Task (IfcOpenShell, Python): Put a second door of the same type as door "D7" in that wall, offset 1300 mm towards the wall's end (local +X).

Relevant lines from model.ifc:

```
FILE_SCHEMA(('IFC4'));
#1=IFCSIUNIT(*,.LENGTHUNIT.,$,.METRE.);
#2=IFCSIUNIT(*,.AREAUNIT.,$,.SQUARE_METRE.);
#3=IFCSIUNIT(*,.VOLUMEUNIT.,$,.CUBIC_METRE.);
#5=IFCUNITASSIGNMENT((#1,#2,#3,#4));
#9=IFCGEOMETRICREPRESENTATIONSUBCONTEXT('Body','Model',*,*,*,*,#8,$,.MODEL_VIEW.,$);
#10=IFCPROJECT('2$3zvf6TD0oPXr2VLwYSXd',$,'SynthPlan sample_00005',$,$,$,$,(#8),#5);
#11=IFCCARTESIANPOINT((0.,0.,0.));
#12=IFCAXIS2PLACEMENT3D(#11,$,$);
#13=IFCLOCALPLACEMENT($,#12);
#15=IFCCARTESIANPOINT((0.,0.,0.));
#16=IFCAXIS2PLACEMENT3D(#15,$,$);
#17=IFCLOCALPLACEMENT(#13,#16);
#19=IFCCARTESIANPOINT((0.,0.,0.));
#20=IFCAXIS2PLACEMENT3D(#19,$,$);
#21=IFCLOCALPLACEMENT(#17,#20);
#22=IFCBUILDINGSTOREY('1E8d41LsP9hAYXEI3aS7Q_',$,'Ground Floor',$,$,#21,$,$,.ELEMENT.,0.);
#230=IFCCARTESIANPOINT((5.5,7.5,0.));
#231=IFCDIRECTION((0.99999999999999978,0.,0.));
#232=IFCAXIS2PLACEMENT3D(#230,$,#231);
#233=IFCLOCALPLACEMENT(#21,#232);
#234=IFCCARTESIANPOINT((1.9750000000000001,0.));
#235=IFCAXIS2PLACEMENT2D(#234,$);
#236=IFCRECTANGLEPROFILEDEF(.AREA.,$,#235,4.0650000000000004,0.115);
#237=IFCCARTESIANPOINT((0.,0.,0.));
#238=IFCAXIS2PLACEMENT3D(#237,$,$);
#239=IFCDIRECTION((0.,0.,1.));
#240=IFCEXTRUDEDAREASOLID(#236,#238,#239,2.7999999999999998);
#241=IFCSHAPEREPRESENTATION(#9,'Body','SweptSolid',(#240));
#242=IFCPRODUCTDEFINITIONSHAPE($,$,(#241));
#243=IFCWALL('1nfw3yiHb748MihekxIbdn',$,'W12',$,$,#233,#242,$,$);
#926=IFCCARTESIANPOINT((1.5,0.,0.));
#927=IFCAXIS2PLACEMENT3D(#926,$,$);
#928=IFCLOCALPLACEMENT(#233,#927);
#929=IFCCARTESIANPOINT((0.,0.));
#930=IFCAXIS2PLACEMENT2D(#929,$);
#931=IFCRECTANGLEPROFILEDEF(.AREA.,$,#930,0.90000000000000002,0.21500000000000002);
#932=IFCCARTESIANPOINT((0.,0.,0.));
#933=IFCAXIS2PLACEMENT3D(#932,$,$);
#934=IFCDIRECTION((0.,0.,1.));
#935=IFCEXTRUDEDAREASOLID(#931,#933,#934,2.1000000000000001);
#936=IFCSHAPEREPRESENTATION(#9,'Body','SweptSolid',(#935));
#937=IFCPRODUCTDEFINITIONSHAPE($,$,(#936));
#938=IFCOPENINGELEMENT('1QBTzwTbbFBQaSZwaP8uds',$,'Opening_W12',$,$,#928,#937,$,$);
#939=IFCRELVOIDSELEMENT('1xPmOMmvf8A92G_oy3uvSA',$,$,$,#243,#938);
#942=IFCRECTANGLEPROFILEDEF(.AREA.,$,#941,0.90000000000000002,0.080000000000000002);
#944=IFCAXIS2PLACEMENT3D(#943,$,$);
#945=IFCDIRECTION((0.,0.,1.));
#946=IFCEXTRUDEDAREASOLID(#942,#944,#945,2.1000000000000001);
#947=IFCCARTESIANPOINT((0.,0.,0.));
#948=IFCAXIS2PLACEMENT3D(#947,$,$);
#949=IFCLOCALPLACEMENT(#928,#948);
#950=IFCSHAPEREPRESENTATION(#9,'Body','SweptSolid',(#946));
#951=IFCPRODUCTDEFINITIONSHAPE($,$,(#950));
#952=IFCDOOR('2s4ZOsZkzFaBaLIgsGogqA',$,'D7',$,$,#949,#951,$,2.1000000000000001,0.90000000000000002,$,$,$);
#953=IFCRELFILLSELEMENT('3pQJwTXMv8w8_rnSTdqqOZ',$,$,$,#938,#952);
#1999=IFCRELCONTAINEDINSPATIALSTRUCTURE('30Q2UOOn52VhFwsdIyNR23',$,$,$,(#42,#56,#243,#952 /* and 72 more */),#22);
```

```python
import ifcopenshell
import ifcopenshell.api.feature
import ifcopenshell.api.geometry
import ifcopenshell.api.root
import ifcopenshell.geom
import ifcopenshell.util.element
import ifcopenshell.util.placement
import ifcopenshell.util.shape
import ifcopenshell.util.unit

model = ifcopenshell.open("model.ifc")
unit_scale = ifcopenshell.util.unit.calculate_unit_scale(model)
settings = ifcopenshell.geom.settings()


def volume(element):
    """Net volume in cubic metres, openings subtracted."""
    shape = ifcopenshell.geom.create_shape(settings, element)
    return ifcopenshell.util.shape.get_volume(shape.geometry)


door = model.by_guid("2s4ZOsZkzFaBaLIgsGogqA")
opening = door.FillsVoids[0].RelatingOpeningElement
wall = opening.VoidsElements[0].RelatingBuildingElement
before = volume(wall)
shift = ifcopenshell.util.placement.get_local_placement(wall.ObjectPlacement)[:3, 0] * 1.3 / unit_scale

# copy_class copies the void relationship, type, container and properties, but no geometry.
new_opening = ifcopenshell.api.root.copy_class(model, product=opening)
new_opening.Representation = ifcopenshell.util.element.copy_deep(
    model, opening.Representation, exclude=["IfcGeometricRepresentationContext", "IfcRepresentationMap"]
)
new_door = ifcopenshell.api.root.copy_class(model, product=door)
new_door.Representation = ifcopenshell.util.element.copy_deep(
    model, door.Representation, exclude=["IfcGeometricRepresentationContext", "IfcRepresentationMap"]
)
ifcopenshell.api.feature.add_filling(model, opening=new_opening, element=new_door)

for old, new in ((opening, new_opening), (door, new_door)):
    matrix = ifcopenshell.util.placement.get_local_placement(old.ObjectPlacement)
    matrix[:3, 3] += shift
    ifcopenshell.api.geometry.edit_object_placement(model, product=new, matrix=matrix, is_si=False)

after = volume(wall)

print(f"wall volume {before:.3f} -> {after:.3f} m3")

model.write("model-out.ifc")
```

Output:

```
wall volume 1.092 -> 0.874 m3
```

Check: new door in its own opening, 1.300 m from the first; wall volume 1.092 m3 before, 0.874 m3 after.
